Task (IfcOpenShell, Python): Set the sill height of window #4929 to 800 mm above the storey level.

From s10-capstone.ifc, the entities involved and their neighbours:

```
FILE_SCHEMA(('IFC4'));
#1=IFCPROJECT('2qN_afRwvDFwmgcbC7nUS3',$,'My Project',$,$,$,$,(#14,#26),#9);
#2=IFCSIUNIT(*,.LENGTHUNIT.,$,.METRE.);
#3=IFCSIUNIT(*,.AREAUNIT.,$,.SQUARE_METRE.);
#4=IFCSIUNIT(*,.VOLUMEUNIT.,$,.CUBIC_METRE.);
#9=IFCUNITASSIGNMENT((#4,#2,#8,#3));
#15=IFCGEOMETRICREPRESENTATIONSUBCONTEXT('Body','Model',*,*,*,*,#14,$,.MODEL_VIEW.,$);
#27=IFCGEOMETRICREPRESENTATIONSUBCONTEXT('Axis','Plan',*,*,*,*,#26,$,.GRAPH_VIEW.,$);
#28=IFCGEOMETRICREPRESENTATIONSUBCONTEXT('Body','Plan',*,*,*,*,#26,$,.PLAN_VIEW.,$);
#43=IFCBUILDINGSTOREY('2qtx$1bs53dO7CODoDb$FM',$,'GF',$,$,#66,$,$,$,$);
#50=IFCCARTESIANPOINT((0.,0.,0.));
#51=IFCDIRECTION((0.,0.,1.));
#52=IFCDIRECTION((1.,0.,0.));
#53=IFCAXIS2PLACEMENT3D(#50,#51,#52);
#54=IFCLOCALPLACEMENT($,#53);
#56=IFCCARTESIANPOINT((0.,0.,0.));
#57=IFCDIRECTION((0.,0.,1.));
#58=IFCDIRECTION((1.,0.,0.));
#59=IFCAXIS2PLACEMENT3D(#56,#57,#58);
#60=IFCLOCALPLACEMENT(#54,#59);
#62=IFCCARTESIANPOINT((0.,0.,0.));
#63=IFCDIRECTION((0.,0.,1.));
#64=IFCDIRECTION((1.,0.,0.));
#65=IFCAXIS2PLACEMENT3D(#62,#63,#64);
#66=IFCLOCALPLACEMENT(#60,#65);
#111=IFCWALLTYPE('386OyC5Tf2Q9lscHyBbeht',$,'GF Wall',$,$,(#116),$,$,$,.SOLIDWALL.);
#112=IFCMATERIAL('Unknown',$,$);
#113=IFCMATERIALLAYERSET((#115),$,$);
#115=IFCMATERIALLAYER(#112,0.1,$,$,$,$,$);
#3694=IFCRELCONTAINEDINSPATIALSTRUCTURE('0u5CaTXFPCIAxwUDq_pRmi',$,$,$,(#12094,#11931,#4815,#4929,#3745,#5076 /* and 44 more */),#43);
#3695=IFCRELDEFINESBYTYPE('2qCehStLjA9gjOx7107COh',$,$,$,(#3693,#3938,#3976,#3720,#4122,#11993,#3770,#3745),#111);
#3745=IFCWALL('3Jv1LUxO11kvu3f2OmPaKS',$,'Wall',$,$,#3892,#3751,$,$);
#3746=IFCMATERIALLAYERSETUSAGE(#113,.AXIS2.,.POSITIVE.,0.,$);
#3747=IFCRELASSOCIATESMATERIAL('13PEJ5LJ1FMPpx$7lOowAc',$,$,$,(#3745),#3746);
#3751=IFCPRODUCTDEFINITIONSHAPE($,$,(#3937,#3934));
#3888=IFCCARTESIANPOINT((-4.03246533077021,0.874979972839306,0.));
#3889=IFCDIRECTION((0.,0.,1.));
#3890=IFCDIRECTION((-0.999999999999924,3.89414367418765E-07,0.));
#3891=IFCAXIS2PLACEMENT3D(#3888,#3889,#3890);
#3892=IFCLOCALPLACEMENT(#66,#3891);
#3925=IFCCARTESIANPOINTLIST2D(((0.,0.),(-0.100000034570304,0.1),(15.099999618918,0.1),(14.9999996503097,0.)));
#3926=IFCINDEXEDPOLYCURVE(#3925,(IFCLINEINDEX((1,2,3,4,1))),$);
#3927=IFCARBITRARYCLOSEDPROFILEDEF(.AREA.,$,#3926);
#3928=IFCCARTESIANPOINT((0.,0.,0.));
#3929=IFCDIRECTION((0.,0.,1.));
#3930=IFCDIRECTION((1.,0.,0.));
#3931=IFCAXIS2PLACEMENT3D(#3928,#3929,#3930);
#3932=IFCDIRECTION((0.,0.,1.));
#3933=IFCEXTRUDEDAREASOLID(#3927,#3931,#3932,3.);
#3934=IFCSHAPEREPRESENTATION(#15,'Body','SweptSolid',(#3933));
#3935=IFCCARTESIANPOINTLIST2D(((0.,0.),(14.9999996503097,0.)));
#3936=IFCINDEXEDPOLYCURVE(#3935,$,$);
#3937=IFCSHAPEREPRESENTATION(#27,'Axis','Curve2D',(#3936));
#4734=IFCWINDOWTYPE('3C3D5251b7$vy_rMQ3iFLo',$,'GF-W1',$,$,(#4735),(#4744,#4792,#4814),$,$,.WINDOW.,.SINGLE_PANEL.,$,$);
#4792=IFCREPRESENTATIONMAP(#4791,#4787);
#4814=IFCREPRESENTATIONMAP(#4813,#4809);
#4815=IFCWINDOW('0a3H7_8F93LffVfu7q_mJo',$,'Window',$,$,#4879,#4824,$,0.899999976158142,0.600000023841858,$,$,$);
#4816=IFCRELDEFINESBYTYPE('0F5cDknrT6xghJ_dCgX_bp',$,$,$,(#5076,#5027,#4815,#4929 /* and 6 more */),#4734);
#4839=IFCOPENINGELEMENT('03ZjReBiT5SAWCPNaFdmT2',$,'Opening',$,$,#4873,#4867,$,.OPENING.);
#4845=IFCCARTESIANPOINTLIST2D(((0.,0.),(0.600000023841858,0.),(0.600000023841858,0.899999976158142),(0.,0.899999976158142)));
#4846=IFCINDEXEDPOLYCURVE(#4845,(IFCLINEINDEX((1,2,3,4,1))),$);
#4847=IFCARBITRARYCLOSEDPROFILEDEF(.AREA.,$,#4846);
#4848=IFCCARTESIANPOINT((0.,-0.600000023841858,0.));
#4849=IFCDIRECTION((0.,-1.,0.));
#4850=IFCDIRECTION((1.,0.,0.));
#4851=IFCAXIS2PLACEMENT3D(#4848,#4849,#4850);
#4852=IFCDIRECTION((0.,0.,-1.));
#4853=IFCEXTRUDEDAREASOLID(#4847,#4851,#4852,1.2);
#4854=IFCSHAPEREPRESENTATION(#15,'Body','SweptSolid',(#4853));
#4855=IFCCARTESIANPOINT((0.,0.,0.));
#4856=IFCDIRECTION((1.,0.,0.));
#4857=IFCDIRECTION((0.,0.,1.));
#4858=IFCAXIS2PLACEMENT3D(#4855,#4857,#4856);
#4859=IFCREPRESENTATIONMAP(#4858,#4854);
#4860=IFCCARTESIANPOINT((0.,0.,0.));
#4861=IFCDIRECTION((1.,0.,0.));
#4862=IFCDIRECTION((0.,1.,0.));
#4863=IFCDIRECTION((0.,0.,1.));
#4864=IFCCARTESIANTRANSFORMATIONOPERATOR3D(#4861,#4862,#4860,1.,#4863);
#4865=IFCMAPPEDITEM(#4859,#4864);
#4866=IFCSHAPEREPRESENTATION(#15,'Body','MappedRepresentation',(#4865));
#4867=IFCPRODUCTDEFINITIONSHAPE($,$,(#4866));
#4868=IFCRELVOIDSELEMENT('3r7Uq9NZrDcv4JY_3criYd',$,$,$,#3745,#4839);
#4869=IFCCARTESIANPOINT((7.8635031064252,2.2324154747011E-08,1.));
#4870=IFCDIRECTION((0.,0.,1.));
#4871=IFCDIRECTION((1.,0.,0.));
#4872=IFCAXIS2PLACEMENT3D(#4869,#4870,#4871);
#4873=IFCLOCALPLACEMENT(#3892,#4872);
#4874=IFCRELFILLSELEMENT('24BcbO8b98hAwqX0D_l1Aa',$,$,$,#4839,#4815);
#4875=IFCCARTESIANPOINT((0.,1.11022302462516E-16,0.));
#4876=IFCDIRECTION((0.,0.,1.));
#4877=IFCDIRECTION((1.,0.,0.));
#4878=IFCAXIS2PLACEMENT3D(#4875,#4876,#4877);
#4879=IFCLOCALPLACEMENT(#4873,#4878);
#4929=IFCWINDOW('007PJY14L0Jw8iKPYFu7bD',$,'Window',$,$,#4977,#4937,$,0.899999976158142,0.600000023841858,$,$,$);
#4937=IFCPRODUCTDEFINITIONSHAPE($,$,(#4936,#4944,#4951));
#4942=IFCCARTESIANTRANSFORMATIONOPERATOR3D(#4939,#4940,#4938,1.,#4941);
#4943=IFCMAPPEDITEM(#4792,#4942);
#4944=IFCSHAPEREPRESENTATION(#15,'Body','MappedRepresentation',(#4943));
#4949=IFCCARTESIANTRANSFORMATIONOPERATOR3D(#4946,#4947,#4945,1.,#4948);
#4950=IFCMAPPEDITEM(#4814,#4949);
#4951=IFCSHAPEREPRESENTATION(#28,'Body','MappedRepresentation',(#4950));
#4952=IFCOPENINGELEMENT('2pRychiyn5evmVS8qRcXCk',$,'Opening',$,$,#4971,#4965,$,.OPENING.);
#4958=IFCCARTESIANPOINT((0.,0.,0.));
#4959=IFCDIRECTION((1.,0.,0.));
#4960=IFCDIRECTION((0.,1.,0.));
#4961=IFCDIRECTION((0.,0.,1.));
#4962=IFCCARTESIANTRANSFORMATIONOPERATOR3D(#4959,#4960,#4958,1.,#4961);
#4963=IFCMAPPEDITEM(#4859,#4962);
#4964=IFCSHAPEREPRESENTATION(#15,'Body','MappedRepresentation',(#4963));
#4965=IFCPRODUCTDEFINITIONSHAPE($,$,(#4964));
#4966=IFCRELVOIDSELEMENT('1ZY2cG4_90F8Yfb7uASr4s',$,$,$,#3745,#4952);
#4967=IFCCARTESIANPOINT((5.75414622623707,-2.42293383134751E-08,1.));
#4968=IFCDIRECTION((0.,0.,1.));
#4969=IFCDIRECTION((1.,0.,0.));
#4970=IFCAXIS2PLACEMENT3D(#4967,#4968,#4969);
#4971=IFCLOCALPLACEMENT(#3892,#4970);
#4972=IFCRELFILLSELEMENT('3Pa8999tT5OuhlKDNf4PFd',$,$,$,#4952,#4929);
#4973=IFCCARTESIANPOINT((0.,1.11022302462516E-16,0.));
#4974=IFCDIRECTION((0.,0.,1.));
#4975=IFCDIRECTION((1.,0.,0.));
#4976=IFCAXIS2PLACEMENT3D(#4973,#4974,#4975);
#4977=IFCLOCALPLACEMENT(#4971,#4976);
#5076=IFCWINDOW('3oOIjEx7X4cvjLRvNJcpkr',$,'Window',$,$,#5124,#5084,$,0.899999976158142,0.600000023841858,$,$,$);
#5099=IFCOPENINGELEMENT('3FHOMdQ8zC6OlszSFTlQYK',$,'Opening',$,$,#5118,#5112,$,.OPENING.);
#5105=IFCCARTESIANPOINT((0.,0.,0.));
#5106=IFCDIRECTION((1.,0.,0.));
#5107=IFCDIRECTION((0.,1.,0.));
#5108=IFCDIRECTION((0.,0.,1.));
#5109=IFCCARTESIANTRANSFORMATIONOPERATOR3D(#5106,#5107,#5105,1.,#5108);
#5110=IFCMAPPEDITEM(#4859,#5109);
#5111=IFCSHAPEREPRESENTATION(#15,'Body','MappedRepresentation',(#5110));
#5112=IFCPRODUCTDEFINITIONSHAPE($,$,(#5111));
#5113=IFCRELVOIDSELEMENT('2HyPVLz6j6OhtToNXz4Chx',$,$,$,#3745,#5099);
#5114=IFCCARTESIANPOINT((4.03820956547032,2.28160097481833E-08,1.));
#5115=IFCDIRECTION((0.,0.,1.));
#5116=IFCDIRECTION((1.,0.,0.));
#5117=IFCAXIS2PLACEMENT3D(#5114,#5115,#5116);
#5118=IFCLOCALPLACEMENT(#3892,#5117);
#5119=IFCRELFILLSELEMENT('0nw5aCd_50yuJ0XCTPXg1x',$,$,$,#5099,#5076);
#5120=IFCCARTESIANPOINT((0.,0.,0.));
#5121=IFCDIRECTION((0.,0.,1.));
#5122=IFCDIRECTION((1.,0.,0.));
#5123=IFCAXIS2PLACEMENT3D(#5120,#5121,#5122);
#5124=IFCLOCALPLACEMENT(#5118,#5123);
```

```python
import numpy as np
import ifcopenshell
import ifcopenshell.api.geometry
import ifcopenshell.geom
import ifcopenshell.util.element
import ifcopenshell.util.placement
import ifcopenshell.util.shape
import ifcopenshell.util.unit

model = ifcopenshell.open("s10-capstone.ifc")
unit_scale = ifcopenshell.util.unit.calculate_unit_scale(model)

window = model.by_guid("007PJY14L0Jw8iKPYFu7bD")
opening = window.FillsVoids[0].RelatingOpeningElement
storey = ifcopenshell.util.element.get_container(window, ifc_class="IfcBuildingStorey")
level = ifcopenshell.util.placement.get_local_placement(storey.ObjectPlacement)[2, 3]

# The opening's origin need not be at the sill, so measure its lowest point.
shape = ifcopenshell.geom.create_shape(ifcopenshell.geom.settings(), opening)
bottom = ifcopenshell.util.shape.get_shape_bottom_elevation(shape, shape.geometry) / unit_scale
dz = level + 0.8 / unit_scale - bottom

shift = np.array([0.0, 0.0, dz])
# The window is placed relative to its opening, so it follows when the opening moves.
matrix = ifcopenshell.util.placement.get_local_placement(opening.ObjectPlacement)
matrix[:3, 3] += shift
ifcopenshell.api.geometry.edit_object_placement(
    model, product=opening, matrix=matrix, is_si=False, should_transform_children=True
)

print(f"moved by {dz * unit_scale:+.3f} m")

model.write("s10-capstone_edited.ifc")
```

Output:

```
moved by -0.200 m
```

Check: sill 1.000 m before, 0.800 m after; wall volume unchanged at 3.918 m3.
